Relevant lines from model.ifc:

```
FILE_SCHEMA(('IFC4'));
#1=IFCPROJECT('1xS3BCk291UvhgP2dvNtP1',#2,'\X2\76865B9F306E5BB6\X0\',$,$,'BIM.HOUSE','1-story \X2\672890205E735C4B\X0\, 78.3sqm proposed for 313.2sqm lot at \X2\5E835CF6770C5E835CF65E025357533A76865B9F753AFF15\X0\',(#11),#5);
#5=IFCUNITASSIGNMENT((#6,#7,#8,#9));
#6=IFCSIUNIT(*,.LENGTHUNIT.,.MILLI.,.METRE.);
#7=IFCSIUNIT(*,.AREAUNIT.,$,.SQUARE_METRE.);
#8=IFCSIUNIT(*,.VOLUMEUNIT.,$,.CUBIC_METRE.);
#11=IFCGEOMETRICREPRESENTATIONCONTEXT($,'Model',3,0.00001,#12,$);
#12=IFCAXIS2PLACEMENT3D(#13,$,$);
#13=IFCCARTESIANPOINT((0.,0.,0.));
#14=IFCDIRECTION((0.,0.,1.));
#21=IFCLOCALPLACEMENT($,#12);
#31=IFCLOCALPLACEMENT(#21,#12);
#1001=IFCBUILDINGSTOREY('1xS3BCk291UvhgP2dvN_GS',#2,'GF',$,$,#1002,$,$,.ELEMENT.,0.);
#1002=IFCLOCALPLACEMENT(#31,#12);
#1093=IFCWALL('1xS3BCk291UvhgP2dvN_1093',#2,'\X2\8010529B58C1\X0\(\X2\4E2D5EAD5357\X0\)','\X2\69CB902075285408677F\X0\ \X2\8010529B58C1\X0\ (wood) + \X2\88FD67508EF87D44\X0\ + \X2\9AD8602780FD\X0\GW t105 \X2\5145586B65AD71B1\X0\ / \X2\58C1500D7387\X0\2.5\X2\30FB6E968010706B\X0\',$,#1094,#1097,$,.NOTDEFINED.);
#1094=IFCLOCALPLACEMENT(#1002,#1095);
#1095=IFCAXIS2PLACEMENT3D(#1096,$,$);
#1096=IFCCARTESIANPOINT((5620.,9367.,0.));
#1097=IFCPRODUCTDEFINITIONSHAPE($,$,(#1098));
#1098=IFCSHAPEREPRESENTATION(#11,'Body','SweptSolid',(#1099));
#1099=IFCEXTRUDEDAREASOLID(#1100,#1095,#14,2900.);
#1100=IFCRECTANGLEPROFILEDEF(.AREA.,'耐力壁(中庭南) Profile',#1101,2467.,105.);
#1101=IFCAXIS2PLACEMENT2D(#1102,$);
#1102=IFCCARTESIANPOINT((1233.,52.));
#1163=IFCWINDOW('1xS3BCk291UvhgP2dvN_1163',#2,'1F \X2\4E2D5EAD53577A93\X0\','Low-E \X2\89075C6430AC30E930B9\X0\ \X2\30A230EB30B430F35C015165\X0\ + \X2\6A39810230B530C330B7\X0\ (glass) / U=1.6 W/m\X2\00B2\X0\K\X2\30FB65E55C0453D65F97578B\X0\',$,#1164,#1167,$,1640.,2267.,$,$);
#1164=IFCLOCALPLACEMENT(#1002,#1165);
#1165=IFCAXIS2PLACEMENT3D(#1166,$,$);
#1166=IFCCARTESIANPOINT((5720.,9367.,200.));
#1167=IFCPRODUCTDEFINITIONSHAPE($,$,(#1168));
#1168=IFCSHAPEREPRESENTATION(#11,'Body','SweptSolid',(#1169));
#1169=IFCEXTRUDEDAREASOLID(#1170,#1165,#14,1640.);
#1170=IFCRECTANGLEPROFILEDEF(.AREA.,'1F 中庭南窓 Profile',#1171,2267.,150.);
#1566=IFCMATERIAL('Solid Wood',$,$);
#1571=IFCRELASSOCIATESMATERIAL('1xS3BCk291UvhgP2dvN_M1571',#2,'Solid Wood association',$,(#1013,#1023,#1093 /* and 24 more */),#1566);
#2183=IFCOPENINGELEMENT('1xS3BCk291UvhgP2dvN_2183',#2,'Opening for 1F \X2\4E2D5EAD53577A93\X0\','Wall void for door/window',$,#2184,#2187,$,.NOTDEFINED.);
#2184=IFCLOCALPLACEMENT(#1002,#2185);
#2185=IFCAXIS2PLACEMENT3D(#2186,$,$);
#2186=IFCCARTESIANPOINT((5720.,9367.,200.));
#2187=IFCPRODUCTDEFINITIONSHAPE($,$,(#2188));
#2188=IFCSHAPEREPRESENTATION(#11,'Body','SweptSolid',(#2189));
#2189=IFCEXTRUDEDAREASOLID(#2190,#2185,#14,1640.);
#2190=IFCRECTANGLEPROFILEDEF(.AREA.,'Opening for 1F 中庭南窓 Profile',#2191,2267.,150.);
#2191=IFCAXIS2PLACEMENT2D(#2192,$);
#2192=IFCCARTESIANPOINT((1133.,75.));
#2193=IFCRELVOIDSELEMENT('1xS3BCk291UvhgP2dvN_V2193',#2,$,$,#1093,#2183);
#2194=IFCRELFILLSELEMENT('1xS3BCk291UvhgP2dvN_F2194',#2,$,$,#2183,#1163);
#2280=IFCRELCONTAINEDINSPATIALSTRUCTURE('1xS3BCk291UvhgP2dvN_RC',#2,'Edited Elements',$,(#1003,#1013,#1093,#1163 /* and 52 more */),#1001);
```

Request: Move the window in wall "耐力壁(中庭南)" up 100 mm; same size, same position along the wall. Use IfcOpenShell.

```python
import numpy as np
import ifcopenshell
import ifcopenshell.api.geometry
import ifcopenshell.util.placement
import ifcopenshell.util.unit

model = ifcopenshell.open("model.ifc")
unit_scale = ifcopenshell.util.unit.calculate_unit_scale(model)

window = model.by_guid("1xS3BCk291UvhgP2dvN_1163")
opening = window.FillsVoids[0].RelatingOpeningElement
dz = 100.0

shift = np.array([0.0, 0.0, dz])
# The window is not placed relative to its opening, so move both.
for product in (opening, window):
    matrix = ifcopenshell.util.placement.get_local_placement(product.ObjectPlacement)
    matrix[:3, 3] += shift
    ifcopenshell.api.geometry.edit_object_placement(model, product=product, matrix=matrix, is_si=False)

print(f"moved by {dz * unit_scale:+.3f} m")

model.write("model_updated.ifc")
```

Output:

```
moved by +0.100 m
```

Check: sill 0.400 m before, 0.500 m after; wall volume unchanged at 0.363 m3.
